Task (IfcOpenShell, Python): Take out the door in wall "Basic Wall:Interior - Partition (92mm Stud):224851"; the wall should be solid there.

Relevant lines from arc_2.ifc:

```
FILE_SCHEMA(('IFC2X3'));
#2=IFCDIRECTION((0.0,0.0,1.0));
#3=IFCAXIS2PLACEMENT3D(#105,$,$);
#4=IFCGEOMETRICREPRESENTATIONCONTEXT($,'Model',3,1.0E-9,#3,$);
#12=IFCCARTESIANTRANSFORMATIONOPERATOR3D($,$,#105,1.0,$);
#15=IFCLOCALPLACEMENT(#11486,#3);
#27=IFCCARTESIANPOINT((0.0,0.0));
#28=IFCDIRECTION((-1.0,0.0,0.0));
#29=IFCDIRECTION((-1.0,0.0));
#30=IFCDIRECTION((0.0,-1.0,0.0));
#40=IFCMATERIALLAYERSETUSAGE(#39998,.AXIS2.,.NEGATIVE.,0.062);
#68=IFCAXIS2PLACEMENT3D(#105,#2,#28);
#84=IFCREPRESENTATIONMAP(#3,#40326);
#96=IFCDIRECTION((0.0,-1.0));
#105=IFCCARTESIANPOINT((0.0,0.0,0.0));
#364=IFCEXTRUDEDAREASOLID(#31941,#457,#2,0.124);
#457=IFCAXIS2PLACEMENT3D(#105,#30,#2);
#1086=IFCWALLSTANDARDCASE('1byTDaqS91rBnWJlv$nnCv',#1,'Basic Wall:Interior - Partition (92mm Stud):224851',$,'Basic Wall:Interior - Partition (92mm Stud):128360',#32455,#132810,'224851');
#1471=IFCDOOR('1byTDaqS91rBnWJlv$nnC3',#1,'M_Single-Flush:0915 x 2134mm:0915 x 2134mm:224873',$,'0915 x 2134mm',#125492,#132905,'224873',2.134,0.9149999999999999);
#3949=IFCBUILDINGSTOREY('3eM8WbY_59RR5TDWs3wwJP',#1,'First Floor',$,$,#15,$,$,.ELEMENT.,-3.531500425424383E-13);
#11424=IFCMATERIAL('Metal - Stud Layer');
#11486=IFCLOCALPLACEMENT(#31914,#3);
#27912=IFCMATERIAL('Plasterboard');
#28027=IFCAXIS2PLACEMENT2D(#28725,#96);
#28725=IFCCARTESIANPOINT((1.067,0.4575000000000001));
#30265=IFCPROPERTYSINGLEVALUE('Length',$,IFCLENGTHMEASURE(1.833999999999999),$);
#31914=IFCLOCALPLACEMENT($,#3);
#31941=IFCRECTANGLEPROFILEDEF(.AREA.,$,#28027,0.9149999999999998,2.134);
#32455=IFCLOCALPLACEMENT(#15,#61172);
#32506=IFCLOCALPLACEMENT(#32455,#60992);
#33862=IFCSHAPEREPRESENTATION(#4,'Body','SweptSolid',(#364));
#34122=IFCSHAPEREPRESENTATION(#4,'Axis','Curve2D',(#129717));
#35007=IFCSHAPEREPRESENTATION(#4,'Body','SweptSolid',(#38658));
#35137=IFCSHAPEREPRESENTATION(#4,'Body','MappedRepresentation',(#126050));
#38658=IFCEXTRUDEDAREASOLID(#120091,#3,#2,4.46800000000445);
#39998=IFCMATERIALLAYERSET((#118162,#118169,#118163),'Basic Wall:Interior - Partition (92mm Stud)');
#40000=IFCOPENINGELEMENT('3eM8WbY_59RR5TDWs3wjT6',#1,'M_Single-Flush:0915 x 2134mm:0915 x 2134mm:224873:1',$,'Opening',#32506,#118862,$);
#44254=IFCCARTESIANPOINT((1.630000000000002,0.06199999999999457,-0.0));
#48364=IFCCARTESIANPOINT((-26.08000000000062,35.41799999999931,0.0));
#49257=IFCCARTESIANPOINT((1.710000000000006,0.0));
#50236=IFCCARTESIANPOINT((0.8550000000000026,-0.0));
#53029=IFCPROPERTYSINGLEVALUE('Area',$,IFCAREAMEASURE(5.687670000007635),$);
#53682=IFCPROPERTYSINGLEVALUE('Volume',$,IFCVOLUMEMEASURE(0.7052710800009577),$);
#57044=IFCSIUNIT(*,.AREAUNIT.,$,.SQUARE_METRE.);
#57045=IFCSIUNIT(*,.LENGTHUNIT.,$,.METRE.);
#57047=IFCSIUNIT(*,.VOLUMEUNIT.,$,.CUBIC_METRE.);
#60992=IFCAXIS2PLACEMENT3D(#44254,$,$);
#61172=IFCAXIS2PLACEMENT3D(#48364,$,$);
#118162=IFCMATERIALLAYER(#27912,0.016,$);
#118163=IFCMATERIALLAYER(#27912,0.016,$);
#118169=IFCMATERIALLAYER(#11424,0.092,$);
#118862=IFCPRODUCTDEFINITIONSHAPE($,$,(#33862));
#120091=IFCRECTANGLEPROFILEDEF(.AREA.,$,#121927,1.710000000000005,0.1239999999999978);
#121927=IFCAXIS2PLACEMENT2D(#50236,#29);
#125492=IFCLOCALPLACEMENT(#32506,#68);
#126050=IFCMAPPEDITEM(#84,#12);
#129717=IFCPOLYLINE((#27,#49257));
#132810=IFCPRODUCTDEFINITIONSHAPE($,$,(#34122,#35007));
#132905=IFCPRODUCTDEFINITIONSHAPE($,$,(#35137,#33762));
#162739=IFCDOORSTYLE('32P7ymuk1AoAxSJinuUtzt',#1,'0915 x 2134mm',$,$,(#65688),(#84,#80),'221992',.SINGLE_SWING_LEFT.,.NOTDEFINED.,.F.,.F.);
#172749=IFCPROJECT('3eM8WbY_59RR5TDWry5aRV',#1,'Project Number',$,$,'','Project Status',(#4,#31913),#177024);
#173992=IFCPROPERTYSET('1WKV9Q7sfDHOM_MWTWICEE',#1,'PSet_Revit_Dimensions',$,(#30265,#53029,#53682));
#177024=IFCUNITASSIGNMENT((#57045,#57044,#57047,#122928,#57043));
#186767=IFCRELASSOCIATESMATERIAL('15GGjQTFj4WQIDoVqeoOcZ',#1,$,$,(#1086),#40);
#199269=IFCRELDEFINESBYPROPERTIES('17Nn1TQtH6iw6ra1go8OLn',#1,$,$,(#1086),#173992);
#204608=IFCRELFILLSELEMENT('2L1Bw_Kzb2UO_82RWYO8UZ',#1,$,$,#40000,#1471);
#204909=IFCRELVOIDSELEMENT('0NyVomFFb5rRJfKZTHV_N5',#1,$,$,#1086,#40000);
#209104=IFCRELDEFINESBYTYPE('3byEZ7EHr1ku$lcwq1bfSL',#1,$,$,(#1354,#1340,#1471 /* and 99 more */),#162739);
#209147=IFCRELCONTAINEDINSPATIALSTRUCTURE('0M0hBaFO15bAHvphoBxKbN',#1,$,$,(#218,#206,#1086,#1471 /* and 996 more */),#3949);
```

```python
import ifcopenshell
import ifcopenshell.api.feature
import ifcopenshell.api.pset
import ifcopenshell.api.root
import ifcopenshell.geom
import ifcopenshell.util.element
import ifcopenshell.util.shape
import ifcopenshell.util.unit

model = ifcopenshell.open("arc_2.ifc")
area_scale = ifcopenshell.util.unit.calculate_unit_scale(model, "AREAUNIT")
volume_scale = ifcopenshell.util.unit.calculate_unit_scale(model, "VOLUMEUNIT")
settings = ifcopenshell.geom.settings()


def volume(element):
    """Net volume in cubic metres, openings subtracted."""
    shape = ifcopenshell.geom.create_shape(settings, element)
    return ifcopenshell.util.shape.get_volume(shape.geometry)


door = model.by_guid("1byTDaqS91rBnWJlv$nnC3")
opening = door.FillsVoids[0].RelatingOpeningElement
wall = opening.VoidsElements[0].RelatingBuildingElement
before = volume(wall)

ifcopenshell.api.root.remove_product(model, product=door)
ifcopenshell.api.feature.remove_feature(model, feature=opening)

after = volume(wall)
thickness = 0.124  # wall thickness in metres

# Update the wall's stored quantities.
pset = model.by_id(ifcopenshell.util.element.get_pset(wall, "PSet_Revit_Dimensions", should_inherit=False)["id"])
ifcopenshell.api.pset.edit_pset(model, pset=pset, properties={
    "Area": model.create_entity("IfcAreaMeasure", after / thickness / area_scale),
    "Volume": model.create_entity("IfcVolumeMeasure", after / volume_scale),
})

print(f"wall volume {before:.3f} -> {after:.3f} m3")

model.write("arc_2-out.ifc")
```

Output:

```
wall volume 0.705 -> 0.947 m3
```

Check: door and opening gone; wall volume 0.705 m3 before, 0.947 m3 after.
